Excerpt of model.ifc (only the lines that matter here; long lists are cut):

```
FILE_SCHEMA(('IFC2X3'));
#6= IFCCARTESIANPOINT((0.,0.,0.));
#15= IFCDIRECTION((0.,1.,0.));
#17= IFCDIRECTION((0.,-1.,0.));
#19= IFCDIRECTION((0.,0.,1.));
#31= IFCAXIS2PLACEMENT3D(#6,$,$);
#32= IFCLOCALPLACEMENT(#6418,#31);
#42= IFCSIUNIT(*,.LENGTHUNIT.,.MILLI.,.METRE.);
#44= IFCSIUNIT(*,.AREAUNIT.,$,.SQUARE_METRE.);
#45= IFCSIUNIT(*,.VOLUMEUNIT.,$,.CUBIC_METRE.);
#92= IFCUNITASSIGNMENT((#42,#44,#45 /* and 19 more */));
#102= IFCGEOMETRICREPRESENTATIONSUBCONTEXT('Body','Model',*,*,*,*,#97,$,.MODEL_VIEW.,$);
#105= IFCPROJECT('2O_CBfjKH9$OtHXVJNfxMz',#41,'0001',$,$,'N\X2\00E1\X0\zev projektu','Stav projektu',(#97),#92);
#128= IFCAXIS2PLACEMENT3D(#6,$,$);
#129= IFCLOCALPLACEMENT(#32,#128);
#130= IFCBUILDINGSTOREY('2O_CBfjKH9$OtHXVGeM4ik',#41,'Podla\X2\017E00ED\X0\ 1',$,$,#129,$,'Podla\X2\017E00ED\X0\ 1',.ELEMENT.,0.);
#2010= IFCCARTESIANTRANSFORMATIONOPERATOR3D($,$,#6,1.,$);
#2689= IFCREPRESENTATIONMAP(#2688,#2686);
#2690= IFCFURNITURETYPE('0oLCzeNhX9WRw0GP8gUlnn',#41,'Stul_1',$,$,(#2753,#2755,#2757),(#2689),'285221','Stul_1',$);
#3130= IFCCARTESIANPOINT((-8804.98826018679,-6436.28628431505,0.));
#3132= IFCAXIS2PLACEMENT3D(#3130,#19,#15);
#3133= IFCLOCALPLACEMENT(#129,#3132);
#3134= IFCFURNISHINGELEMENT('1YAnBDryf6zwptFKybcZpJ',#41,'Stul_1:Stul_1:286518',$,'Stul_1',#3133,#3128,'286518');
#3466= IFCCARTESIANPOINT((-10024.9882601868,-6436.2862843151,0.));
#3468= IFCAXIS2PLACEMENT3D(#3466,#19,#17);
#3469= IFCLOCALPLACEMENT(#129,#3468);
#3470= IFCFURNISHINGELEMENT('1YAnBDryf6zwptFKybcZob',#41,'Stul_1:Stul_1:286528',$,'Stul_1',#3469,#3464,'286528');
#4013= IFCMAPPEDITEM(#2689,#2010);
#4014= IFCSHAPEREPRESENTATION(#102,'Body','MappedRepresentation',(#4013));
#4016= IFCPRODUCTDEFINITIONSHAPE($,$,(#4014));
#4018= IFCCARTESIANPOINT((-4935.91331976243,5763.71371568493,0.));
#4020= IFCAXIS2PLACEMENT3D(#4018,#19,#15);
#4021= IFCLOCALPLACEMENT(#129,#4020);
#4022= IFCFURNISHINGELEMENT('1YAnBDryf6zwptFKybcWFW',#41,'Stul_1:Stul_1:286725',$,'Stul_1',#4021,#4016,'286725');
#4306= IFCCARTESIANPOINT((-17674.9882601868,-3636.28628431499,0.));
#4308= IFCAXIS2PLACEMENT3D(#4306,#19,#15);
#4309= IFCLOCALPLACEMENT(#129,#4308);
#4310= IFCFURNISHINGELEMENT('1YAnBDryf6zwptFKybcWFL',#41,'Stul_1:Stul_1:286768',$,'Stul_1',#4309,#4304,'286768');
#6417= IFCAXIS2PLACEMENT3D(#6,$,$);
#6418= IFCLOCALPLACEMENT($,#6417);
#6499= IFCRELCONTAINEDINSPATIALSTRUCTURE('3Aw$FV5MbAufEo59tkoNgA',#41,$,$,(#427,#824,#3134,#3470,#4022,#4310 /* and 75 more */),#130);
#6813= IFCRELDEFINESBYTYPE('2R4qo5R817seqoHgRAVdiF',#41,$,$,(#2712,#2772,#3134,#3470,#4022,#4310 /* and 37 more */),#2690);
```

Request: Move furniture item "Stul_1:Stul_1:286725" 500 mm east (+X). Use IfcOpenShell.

```python
import ifcopenshell
import ifcopenshell.api.geometry
import ifcopenshell.util.placement

model = ifcopenshell.open("model.ifc")

item = model.by_guid("1YAnBDryf6zwptFKybcWFW")
matrix = ifcopenshell.util.placement.get_local_placement(item.ObjectPlacement)
matrix[0, 3] += 500.0
ifcopenshell.api.geometry.edit_object_placement(model, product=item, matrix=matrix, is_si=False)

print(ifcopenshell.util.placement.get_local_placement(item.ObjectPlacement).round(3) + 0.0)

model.write("model_v2.ifc")
```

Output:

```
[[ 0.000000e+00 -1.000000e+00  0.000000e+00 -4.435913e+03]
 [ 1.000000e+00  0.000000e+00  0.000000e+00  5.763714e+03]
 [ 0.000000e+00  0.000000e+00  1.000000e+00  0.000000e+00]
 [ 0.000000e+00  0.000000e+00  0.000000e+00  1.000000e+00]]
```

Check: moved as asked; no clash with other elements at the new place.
